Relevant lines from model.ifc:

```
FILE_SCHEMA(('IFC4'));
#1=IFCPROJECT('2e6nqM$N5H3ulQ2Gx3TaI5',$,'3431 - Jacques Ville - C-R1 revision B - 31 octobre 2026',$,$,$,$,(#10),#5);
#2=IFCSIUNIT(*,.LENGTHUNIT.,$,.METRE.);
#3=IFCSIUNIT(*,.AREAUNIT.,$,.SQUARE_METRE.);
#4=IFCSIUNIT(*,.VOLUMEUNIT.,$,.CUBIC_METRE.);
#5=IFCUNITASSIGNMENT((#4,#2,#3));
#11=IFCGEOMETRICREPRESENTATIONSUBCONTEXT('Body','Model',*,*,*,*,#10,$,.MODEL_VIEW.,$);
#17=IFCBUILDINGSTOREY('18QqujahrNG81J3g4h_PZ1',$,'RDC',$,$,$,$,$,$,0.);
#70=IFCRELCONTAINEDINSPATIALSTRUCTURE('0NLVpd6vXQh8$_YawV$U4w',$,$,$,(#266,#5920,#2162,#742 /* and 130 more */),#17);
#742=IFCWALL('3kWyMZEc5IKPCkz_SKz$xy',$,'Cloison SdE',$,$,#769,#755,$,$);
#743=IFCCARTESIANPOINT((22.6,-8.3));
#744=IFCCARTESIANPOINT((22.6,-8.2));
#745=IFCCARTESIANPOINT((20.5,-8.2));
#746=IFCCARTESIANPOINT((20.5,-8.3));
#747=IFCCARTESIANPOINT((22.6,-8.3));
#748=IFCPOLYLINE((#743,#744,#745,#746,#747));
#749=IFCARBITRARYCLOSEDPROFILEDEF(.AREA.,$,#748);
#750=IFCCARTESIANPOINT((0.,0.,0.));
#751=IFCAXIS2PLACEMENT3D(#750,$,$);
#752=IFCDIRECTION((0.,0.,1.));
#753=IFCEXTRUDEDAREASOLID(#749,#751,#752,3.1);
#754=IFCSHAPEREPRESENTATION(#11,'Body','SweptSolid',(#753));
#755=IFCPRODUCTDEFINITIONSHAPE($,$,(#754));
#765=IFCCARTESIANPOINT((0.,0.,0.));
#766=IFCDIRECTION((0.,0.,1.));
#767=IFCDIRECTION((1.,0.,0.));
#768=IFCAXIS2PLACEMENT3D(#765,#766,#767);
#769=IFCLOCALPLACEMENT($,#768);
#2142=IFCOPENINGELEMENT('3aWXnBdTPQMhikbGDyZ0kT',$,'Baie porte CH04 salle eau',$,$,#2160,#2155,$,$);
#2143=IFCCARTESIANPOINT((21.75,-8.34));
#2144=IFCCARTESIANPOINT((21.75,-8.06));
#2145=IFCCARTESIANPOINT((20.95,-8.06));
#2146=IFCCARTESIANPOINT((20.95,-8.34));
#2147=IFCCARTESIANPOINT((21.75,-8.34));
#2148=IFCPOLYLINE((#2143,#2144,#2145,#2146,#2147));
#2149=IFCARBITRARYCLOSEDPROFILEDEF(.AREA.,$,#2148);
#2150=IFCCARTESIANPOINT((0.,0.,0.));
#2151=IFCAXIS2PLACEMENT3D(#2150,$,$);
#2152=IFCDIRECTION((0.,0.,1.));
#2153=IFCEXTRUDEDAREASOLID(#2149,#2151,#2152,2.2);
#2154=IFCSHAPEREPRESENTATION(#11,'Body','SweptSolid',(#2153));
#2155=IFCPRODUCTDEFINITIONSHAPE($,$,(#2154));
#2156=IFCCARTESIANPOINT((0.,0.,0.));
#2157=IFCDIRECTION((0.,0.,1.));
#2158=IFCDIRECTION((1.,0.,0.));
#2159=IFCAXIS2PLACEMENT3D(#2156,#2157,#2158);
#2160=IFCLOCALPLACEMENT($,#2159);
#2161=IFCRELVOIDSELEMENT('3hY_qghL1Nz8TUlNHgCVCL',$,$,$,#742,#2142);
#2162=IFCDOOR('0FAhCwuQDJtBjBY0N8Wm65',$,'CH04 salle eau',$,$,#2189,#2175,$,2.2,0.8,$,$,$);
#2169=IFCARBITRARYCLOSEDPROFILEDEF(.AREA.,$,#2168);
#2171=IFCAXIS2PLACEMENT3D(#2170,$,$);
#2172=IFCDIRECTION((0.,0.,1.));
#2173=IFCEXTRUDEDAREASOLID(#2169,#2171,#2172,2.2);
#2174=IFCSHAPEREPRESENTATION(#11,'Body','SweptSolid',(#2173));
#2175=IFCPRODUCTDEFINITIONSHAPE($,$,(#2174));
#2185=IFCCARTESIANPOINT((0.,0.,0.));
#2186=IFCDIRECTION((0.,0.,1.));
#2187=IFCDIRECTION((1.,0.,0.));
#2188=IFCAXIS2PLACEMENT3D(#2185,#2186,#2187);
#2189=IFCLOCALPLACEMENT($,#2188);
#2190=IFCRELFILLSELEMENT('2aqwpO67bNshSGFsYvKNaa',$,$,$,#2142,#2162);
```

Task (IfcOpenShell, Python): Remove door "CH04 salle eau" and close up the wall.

```python
import ifcopenshell
import ifcopenshell.api.feature
import ifcopenshell.api.root
import ifcopenshell.geom
import ifcopenshell.util.shape

model = ifcopenshell.open("model.ifc")
settings = ifcopenshell.geom.settings()


def volume(element):
    """Net volume in cubic metres, openings subtracted."""
    shape = ifcopenshell.geom.create_shape(settings, element)
    return ifcopenshell.util.shape.get_volume(shape.geometry)


door = model.by_guid("0FAhCwuQDJtBjBY0N8Wm65")
opening = door.FillsVoids[0].RelatingOpeningElement
wall = opening.VoidsElements[0].RelatingBuildingElement
before = volume(wall)

ifcopenshell.api.root.remove_product(model, product=door)
ifcopenshell.api.feature.remove_feature(model, feature=opening)

after = volume(wall)

print(f"wall volume {before:.3f} -> {after:.3f} m3")

model.write("model-out.ifc")
```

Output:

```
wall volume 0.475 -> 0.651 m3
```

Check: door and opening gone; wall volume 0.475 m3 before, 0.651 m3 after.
